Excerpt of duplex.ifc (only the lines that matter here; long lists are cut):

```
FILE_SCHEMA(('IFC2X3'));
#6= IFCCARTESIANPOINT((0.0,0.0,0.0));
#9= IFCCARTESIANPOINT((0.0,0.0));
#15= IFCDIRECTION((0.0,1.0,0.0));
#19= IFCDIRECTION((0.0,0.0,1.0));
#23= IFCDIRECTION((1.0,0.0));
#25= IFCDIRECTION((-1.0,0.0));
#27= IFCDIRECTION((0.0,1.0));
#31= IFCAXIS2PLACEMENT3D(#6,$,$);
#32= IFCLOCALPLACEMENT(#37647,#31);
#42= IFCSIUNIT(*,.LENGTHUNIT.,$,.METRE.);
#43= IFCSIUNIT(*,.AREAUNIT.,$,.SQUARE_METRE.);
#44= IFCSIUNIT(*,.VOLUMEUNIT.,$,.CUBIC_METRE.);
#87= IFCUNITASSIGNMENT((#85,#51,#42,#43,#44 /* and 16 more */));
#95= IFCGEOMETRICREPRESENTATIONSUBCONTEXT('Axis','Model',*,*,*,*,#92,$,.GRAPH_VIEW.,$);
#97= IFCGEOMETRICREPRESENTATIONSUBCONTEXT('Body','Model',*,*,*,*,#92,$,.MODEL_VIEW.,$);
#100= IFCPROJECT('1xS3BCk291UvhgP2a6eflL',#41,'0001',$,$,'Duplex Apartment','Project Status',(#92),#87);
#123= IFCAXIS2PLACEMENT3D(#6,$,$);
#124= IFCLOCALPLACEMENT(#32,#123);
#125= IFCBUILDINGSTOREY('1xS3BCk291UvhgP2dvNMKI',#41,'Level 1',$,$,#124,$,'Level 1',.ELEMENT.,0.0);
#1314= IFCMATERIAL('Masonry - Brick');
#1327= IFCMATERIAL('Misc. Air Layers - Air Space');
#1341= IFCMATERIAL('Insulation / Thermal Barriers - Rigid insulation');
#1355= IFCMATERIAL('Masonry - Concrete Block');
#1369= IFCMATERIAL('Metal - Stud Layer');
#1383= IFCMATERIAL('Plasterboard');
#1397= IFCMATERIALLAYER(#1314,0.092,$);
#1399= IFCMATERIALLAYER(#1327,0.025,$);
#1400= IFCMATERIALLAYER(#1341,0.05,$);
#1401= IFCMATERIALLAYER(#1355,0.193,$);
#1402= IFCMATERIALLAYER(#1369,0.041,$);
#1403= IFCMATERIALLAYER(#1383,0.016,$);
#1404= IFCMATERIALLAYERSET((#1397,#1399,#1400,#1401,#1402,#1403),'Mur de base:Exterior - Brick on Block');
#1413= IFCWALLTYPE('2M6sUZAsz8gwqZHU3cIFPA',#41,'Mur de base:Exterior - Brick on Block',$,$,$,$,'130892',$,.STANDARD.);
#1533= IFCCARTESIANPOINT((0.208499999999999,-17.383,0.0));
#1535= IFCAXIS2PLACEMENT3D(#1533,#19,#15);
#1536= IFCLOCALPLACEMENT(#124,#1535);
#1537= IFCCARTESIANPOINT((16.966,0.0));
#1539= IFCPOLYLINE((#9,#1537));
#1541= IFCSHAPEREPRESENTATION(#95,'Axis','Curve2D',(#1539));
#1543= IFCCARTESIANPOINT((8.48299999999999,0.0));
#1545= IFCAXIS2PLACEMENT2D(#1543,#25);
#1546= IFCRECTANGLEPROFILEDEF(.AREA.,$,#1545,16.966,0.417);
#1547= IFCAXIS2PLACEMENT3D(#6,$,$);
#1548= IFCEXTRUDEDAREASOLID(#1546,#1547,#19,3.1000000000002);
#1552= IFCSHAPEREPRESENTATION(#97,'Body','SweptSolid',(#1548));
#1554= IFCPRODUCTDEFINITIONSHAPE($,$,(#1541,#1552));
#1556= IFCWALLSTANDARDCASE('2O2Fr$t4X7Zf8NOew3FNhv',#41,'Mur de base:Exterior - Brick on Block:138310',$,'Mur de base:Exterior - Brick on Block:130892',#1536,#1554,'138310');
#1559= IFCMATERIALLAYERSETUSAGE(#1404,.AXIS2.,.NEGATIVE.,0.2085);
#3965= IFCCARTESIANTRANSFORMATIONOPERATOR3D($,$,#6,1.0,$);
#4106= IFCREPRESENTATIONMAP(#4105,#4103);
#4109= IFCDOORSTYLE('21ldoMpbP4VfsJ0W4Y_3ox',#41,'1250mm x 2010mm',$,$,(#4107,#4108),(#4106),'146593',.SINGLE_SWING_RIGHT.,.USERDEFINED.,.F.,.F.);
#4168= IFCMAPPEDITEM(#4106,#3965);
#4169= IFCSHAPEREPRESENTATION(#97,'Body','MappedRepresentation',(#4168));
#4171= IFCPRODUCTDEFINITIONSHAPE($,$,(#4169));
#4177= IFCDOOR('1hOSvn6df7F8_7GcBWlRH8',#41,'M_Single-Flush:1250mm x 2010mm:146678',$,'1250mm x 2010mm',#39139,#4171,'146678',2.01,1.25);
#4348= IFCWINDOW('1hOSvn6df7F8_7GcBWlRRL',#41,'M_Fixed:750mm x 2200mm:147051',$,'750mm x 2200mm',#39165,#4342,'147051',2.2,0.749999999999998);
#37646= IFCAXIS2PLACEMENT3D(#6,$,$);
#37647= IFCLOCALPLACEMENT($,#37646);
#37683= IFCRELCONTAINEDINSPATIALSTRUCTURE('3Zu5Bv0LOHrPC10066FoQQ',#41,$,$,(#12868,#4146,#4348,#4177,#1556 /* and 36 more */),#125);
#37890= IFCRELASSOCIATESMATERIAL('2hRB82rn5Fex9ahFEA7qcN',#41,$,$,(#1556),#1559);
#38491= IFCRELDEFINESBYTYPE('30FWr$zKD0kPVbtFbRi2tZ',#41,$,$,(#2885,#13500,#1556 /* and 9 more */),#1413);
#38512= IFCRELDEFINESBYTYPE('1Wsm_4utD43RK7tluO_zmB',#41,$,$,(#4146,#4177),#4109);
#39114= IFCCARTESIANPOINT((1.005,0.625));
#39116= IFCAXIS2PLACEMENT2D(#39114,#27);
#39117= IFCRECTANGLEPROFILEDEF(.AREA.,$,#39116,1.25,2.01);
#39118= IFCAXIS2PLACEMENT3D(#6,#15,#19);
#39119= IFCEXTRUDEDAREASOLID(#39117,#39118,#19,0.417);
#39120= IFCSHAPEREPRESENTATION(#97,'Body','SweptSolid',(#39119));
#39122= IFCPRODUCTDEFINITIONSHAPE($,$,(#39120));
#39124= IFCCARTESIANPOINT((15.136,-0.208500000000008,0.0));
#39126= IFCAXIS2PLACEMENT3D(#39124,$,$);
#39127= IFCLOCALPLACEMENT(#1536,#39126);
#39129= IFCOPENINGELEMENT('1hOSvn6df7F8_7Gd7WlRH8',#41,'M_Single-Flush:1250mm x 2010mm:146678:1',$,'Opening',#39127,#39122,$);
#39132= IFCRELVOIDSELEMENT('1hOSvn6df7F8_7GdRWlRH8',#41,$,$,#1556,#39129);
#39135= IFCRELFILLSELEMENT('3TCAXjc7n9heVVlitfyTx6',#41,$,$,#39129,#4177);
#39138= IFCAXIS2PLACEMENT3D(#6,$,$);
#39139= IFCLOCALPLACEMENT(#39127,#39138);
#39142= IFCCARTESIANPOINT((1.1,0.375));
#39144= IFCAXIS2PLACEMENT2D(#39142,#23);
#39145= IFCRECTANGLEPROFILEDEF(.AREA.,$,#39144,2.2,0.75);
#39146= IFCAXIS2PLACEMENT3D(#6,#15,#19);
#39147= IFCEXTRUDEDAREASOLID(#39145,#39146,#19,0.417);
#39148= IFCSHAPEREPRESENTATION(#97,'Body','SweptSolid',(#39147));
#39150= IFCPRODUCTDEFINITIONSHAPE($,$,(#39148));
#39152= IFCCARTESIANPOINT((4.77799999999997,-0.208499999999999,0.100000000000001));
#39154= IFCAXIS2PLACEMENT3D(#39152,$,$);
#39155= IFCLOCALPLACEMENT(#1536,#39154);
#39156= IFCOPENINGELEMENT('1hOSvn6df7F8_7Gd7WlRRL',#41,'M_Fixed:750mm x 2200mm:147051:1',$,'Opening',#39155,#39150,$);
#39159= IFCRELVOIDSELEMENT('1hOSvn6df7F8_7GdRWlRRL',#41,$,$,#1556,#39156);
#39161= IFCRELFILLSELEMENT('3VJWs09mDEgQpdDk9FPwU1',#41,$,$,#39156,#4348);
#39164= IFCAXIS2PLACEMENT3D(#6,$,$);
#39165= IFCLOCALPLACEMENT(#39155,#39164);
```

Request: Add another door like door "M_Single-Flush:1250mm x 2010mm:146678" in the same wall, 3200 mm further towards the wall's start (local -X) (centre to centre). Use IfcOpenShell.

```python
import ifcopenshell
import ifcopenshell.api.feature
import ifcopenshell.api.geometry
import ifcopenshell.api.root
import ifcopenshell.geom
import ifcopenshell.util.element
import ifcopenshell.util.placement
import ifcopenshell.util.shape
import ifcopenshell.util.unit

model = ifcopenshell.open("duplex.ifc")
unit_scale = ifcopenshell.util.unit.calculate_unit_scale(model)
settings = ifcopenshell.geom.settings()


def volume(element):
    """Net volume in cubic metres, openings subtracted."""
    shape = ifcopenshell.geom.create_shape(settings, element)
    return ifcopenshell.util.shape.get_volume(shape.geometry)


def reuse_history(source, copy):
    """copy_class also copies each property set's owner history, people and application; keep the originals."""
    for rel in copy.IsDefinedBy:
        if rel.is_a("IfcRelDefinesByProperties") and (history := rel.RelatingPropertyDefinition.OwnerHistory):
            rel.RelatingPropertyDefinition.OwnerHistory = source.OwnerHistory
            ifcopenshell.util.element.remove_deep2(model, history)


door = model.by_guid("1hOSvn6df7F8_7GcBWlRH8")
opening = door.FillsVoids[0].RelatingOpeningElement
wall = opening.VoidsElements[0].RelatingBuildingElement
before = volume(wall)
shift = ifcopenshell.util.placement.get_local_placement(wall.ObjectPlacement)[:3, 0] * -3.2 / unit_scale

# copy_class copies the void relationship, type, container and properties, but no geometry.
new_opening = ifcopenshell.api.root.copy_class(model, product=opening)
new_opening.Representation = ifcopenshell.util.element.copy_deep(
    model, opening.Representation, exclude=["IfcGeometricRepresentationContext", "IfcRepresentationMap"]
)
new_opening.Name = "M_Single-Flush:1250mm x 2010mm"
new_door = ifcopenshell.api.root.copy_class(model, product=door)
new_door.Representation = ifcopenshell.util.element.copy_deep(
    model, door.Representation, exclude=["IfcGeometricRepresentationContext", "IfcRepresentationMap"]
)
new_door.Name = "M_Single-Flush:1250mm x 2010mm"
new_door.Tag = None
reuse_history(door, new_door)
fills = ifcopenshell.api.feature.add_filling(model, opening=new_opening, element=new_door)
fills.OwnerHistory = new_door.OwnerHistory  # required in IFC2X3

for old, new in ((opening, new_opening), (door, new_door)):
    matrix = ifcopenshell.util.placement.get_local_placement(old.ObjectPlacement)
    matrix[:3, 3] += shift
    ifcopenshell.api.geometry.edit_object_placement(model, product=new, matrix=matrix, is_si=False)

after = volume(wall)

print(f"wall volume {before:.3f} -> {after:.3f} m3")

model.write("duplex-out.ifc")
```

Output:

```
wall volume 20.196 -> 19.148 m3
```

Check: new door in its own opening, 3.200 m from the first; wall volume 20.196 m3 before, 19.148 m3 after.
